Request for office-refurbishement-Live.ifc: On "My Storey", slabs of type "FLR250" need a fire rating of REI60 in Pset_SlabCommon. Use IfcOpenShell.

First a look at what the model holds.

```python
import ifcopenshell
import ifcopenshell.util.element

model = ifcopenshell.open("office-refurbishement-Live.ifc")
print(model.schema)
storey = next(s for s in model.by_type("IfcBuildingStorey") if s.Name == "My Storey")
slabs = [e for e in ifcopenshell.util.element.get_decomposition(storey) if e.is_a("IfcSlab")]
seen = {}
for e in slabs:
    element_type = ifcopenshell.util.element.get_type(e)
    key = (element_type.Name if element_type != e and element_type else None, ifcopenshell.util.element.get_pset(e, "Pset_SlabCommon", "FireRating"))
    seen[key] = seen.get(key, 0) + 1
for (name, value), count in sorted(seen.items(), key=str):
    print(count, "x", name, "|", value)
```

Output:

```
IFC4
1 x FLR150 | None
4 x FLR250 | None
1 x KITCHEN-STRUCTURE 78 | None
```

```python
import ifcopenshell
import ifcopenshell.api.pset
import ifcopenshell.util.element

model = ifcopenshell.open("office-refurbishement-Live.ifc")

storey = next(s for s in model.by_type("IfcBuildingStorey") if s.Name == "My Storey")
slabs = [e for e in ifcopenshell.util.element.get_decomposition(storey) if e.is_a("IfcSlab")]

count = 0
for e in slabs:
    element_type = ifcopenshell.util.element.get_type(e)
    if element_type in (None, e) or element_type.Name != "FLR250":
        continue
    # add_pset returns the element's existing set when there is one.
    pset = ifcopenshell.api.pset.add_pset(model, product=e, name="Pset_SlabCommon")
    ifcopenshell.api.pset.edit_pset(model, pset=pset, properties={"FireRating": "REI60"})
    count += 1

print(count, "slabs updated")

model.write("office-refurbishement-Live_edited.ifc")
```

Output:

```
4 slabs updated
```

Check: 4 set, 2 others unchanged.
